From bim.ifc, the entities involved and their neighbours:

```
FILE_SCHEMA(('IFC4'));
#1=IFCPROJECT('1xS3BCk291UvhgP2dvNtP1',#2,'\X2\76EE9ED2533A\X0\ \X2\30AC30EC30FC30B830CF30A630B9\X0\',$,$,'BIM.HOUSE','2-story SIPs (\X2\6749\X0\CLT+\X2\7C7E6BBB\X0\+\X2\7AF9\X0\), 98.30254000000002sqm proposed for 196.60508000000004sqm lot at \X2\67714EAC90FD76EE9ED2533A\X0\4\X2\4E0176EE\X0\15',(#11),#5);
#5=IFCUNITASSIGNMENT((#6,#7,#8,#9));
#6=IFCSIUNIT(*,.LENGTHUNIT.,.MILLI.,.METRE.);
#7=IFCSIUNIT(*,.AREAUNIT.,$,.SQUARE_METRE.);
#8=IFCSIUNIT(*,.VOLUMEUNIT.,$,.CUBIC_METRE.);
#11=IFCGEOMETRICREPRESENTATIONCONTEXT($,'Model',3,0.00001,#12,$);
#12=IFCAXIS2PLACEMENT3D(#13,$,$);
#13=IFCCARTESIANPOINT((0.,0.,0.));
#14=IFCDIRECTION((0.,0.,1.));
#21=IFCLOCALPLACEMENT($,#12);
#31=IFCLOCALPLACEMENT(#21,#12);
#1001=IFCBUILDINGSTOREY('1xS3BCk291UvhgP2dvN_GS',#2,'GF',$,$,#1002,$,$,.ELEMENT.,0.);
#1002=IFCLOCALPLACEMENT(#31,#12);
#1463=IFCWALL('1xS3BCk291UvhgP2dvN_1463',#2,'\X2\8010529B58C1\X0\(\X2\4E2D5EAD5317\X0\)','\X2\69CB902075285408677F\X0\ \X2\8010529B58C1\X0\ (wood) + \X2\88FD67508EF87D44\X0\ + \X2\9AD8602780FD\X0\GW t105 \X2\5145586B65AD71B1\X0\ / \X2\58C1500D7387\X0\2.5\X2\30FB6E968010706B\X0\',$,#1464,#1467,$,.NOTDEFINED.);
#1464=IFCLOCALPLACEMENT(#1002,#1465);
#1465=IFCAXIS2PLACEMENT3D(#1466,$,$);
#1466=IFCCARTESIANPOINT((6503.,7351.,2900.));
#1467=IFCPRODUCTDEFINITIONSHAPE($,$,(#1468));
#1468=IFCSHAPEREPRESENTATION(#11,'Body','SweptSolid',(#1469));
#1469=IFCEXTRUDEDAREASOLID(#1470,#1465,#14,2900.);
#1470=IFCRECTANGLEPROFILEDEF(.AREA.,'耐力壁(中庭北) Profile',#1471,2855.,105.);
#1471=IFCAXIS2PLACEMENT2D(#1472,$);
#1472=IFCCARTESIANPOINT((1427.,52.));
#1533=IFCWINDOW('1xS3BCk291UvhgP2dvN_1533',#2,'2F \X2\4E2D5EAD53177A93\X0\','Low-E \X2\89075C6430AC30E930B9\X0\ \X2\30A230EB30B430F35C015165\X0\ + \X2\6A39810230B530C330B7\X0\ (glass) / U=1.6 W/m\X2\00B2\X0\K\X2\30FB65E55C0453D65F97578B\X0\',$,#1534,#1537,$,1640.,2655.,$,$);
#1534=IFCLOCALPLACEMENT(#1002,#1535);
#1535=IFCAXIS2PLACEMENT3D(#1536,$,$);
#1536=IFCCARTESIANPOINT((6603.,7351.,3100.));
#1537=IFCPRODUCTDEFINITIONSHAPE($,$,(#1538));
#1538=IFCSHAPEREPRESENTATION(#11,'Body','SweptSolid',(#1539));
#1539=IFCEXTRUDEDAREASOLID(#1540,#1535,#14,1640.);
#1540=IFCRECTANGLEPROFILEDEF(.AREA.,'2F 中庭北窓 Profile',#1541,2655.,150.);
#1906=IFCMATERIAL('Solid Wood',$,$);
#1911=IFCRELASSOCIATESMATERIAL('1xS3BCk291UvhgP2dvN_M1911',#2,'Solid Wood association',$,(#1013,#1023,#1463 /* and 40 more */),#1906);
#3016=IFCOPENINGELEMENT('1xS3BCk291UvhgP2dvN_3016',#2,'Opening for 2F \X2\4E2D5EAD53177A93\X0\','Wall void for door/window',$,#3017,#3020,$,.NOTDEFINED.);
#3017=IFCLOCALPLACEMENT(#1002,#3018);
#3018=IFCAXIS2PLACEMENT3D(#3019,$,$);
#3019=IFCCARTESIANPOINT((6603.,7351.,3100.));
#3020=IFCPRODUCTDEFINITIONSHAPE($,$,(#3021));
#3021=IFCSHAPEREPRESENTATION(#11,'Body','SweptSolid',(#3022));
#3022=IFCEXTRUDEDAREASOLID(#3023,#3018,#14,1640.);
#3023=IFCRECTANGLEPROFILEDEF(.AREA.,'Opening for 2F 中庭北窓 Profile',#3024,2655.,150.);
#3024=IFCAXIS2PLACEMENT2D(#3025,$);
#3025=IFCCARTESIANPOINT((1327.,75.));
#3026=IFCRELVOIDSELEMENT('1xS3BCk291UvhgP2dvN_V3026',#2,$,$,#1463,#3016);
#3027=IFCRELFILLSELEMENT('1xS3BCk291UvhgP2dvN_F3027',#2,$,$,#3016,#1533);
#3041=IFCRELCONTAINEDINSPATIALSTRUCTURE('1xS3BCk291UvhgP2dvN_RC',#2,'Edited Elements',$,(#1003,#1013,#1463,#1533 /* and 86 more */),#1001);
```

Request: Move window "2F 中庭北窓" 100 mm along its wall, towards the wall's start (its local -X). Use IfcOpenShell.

```python
import ifcopenshell
import ifcopenshell.api.geometry
import ifcopenshell.util.placement

model = ifcopenshell.open("bim.ifc")

window = model.by_id(1533)
opening = window.FillsVoids[0].RelatingOpeningElement
wall = opening.VoidsElements[0].RelatingBuildingElement

wall_matrix = ifcopenshell.util.placement.get_local_placement(wall.ObjectPlacement)
shift = wall_matrix[:3, 0] * -100.0
before = ifcopenshell.util.placement.get_local_placement(window.ObjectPlacement)[:3, 3].copy()

# The window is not placed relative to its opening, so move both.
for product in (opening, window):
    matrix = ifcopenshell.util.placement.get_local_placement(product.ObjectPlacement)
    matrix[:3, 3] += shift
    ifcopenshell.api.geometry.edit_object_placement(model, product=product, matrix=matrix, is_si=False)

after = ifcopenshell.util.placement.get_local_placement(window.ObjectPlacement)[:3, 3]
print("window moved by", (after - before).round(3) + 0.0)

model.write("bim_v2.ifc")
```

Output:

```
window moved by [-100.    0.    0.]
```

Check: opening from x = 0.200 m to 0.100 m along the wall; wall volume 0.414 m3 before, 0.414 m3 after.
